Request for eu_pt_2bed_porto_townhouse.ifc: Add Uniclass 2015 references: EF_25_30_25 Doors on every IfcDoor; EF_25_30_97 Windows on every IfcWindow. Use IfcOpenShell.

First a look at what the model holds.

```python
import ifcopenshell

model = ifcopenshell.open("eu_pt_2bed_porto_townhouse.ifc")
print(model.schema)
print("classifications:", [c.Name for c in model.by_type("IfcClassification")])
for ifc_class in ("IfcDoor", "IfcRoof", "IfcStair", "IfcWall", "IfcWindow"):
    print(ifc_class, len(model.by_type(ifc_class)))
```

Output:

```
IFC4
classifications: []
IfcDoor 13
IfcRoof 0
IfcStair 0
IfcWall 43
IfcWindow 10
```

```python
import ifcopenshell
import ifcopenshell.api.classification

model = ifcopenshell.open("eu_pt_2bed_porto_townhouse.ifc")

system = ifcopenshell.api.classification.add_classification(model, classification="Uniclass 2015")

codes = {
    "IfcDoor": ("EF_25_30_25", "Doors"),
    "IfcWindow": ("EF_25_30_97", "Windows"),
}
for ifc_class, (code, name) in codes.items():
    products = model.by_type(ifc_class)
    ifcopenshell.api.classification.add_reference(
        model, products=products, classification=system, identification=code, name=name
    )
    print(code, len(products))

model.write("eu_pt_2bed_porto_townhouse_v2.ifc")
```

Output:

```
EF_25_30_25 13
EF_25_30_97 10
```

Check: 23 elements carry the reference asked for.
